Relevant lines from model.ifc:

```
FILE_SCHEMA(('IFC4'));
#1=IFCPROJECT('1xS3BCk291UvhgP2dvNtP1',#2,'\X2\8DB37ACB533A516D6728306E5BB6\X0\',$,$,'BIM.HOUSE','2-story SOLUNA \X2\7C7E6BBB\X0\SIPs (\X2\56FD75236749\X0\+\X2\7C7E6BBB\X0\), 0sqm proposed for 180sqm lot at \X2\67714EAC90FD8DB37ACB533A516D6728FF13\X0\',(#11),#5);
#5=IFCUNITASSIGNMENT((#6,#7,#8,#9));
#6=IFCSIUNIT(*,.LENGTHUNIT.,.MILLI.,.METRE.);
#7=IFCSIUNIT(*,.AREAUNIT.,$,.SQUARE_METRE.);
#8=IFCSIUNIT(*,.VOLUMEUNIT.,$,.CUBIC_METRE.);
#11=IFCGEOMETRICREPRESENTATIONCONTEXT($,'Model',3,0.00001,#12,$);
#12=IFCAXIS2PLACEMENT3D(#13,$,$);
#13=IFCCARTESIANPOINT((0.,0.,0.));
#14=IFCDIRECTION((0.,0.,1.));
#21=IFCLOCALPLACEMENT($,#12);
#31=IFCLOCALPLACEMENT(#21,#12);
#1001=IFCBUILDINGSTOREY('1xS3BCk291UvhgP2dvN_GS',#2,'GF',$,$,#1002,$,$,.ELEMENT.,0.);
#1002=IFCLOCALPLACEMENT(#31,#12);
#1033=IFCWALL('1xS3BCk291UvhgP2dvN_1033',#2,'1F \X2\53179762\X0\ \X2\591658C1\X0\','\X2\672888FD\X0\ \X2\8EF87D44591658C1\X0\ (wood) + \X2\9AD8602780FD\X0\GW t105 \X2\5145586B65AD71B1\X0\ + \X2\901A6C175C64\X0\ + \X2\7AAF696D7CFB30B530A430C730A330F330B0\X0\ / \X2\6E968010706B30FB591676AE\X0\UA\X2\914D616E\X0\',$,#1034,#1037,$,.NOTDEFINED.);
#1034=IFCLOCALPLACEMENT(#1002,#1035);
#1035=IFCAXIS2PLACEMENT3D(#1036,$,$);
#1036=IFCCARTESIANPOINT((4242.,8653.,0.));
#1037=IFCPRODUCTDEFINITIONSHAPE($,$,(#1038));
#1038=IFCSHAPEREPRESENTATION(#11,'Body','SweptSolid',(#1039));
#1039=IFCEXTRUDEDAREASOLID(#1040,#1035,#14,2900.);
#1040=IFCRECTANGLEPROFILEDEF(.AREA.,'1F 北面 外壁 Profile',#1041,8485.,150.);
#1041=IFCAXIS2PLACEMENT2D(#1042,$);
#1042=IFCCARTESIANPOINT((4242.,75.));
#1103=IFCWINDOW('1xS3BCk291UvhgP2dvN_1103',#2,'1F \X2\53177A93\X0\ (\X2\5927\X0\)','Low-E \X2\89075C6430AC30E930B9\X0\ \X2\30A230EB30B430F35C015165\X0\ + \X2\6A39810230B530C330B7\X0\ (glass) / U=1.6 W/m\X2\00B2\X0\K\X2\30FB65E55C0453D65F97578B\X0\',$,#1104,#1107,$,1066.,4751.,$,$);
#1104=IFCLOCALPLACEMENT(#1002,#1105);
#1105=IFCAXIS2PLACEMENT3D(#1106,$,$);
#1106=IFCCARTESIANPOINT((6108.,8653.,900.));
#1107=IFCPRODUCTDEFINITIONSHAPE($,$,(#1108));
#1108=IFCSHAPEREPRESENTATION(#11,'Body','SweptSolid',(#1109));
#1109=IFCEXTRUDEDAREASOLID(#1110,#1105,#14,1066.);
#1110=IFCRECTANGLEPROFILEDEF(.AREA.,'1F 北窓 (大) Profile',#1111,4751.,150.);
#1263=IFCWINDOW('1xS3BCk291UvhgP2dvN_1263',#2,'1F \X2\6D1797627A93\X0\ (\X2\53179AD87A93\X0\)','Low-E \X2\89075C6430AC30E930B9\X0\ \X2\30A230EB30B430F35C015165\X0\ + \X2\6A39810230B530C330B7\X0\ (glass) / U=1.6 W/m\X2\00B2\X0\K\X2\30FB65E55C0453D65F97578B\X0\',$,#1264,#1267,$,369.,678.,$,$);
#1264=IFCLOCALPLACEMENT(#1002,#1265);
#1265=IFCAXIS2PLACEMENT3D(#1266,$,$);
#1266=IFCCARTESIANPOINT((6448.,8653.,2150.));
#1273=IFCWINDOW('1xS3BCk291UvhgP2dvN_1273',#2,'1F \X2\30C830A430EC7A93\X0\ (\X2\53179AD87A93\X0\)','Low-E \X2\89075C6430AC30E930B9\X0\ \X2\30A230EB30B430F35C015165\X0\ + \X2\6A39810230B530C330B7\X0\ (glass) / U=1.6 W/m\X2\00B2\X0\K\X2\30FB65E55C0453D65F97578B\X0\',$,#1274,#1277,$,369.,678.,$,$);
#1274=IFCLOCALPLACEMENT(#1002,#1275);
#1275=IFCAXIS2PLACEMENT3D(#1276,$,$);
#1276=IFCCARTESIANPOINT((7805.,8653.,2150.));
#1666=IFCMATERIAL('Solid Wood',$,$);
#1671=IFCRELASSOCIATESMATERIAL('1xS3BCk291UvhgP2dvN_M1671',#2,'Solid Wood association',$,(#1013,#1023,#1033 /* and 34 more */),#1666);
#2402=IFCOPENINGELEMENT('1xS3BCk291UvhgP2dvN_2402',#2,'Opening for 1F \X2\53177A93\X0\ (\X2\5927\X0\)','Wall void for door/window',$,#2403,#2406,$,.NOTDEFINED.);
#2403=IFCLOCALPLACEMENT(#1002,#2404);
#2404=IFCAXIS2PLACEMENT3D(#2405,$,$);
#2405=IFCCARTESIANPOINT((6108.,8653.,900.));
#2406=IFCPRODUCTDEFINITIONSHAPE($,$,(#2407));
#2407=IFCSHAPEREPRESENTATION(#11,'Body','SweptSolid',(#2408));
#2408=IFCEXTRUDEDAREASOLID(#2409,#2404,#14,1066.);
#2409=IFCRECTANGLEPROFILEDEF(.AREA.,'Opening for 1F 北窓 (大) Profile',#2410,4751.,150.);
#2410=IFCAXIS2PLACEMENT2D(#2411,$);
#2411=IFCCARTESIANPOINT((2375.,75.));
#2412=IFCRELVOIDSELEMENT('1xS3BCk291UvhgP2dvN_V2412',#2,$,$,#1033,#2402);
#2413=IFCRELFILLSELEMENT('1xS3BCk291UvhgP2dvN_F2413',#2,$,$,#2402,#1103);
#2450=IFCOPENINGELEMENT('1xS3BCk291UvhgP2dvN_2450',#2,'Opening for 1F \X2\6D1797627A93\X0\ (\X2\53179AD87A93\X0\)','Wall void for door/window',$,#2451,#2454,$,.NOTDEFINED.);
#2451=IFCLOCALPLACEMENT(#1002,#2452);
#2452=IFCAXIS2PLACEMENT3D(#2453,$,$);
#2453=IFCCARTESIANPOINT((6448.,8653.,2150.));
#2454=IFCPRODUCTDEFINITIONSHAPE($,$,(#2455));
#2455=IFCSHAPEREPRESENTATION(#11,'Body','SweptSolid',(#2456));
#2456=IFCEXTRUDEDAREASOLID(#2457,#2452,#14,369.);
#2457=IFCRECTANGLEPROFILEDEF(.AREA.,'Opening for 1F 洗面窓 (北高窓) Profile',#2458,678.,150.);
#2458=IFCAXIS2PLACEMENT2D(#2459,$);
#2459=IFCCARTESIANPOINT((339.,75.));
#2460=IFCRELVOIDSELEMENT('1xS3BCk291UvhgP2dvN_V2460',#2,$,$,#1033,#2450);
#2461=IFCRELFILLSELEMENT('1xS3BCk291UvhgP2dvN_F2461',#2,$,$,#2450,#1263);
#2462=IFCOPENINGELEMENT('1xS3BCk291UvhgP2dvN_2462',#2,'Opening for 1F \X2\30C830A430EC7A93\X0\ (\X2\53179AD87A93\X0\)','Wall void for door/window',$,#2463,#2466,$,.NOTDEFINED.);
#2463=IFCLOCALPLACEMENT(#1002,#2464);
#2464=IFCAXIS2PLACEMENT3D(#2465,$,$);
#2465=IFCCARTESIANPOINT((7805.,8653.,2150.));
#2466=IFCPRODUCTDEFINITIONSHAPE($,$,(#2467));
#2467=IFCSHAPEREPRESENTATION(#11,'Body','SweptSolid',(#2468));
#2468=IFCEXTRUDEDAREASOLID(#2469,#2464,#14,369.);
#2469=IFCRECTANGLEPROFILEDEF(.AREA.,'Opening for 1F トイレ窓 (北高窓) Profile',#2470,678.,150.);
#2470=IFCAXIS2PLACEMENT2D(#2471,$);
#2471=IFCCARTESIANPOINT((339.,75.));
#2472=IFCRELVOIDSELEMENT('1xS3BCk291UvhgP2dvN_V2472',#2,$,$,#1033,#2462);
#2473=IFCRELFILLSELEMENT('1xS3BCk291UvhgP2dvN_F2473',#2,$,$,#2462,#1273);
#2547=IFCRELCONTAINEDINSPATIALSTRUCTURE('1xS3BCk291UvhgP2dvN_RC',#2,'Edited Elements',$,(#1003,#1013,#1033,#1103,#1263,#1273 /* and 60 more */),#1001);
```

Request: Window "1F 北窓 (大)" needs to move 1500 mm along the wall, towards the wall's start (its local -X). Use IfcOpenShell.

```python
import ifcopenshell
import ifcopenshell.api.geometry
import ifcopenshell.util.placement

model = ifcopenshell.open("model.ifc")

window = model.by_guid("1xS3BCk291UvhgP2dvN_1103")
opening = window.FillsVoids[0].RelatingOpeningElement
wall = opening.VoidsElements[0].RelatingBuildingElement

wall_matrix = ifcopenshell.util.placement.get_local_placement(wall.ObjectPlacement)
shift = wall_matrix[:3, 0] * -1500.0
before = ifcopenshell.util.placement.get_local_placement(window.ObjectPlacement)[:3, 3].copy()

# The window is not placed relative to its opening, so move both.
for product in (opening, window):
    matrix = ifcopenshell.util.placement.get_local_placement(product.ObjectPlacement)
    matrix[:3, 3] += shift
    ifcopenshell.api.geometry.edit_object_placement(model, product=product, matrix=matrix, is_si=False)

after = ifcopenshell.util.placement.get_local_placement(window.ObjectPlacement)[:3, 3]
print("window moved by", (after - before).round(3) + 0.0)

model.write("model_updated.ifc")
```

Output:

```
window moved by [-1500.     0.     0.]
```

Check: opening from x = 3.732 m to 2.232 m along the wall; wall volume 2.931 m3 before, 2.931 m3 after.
